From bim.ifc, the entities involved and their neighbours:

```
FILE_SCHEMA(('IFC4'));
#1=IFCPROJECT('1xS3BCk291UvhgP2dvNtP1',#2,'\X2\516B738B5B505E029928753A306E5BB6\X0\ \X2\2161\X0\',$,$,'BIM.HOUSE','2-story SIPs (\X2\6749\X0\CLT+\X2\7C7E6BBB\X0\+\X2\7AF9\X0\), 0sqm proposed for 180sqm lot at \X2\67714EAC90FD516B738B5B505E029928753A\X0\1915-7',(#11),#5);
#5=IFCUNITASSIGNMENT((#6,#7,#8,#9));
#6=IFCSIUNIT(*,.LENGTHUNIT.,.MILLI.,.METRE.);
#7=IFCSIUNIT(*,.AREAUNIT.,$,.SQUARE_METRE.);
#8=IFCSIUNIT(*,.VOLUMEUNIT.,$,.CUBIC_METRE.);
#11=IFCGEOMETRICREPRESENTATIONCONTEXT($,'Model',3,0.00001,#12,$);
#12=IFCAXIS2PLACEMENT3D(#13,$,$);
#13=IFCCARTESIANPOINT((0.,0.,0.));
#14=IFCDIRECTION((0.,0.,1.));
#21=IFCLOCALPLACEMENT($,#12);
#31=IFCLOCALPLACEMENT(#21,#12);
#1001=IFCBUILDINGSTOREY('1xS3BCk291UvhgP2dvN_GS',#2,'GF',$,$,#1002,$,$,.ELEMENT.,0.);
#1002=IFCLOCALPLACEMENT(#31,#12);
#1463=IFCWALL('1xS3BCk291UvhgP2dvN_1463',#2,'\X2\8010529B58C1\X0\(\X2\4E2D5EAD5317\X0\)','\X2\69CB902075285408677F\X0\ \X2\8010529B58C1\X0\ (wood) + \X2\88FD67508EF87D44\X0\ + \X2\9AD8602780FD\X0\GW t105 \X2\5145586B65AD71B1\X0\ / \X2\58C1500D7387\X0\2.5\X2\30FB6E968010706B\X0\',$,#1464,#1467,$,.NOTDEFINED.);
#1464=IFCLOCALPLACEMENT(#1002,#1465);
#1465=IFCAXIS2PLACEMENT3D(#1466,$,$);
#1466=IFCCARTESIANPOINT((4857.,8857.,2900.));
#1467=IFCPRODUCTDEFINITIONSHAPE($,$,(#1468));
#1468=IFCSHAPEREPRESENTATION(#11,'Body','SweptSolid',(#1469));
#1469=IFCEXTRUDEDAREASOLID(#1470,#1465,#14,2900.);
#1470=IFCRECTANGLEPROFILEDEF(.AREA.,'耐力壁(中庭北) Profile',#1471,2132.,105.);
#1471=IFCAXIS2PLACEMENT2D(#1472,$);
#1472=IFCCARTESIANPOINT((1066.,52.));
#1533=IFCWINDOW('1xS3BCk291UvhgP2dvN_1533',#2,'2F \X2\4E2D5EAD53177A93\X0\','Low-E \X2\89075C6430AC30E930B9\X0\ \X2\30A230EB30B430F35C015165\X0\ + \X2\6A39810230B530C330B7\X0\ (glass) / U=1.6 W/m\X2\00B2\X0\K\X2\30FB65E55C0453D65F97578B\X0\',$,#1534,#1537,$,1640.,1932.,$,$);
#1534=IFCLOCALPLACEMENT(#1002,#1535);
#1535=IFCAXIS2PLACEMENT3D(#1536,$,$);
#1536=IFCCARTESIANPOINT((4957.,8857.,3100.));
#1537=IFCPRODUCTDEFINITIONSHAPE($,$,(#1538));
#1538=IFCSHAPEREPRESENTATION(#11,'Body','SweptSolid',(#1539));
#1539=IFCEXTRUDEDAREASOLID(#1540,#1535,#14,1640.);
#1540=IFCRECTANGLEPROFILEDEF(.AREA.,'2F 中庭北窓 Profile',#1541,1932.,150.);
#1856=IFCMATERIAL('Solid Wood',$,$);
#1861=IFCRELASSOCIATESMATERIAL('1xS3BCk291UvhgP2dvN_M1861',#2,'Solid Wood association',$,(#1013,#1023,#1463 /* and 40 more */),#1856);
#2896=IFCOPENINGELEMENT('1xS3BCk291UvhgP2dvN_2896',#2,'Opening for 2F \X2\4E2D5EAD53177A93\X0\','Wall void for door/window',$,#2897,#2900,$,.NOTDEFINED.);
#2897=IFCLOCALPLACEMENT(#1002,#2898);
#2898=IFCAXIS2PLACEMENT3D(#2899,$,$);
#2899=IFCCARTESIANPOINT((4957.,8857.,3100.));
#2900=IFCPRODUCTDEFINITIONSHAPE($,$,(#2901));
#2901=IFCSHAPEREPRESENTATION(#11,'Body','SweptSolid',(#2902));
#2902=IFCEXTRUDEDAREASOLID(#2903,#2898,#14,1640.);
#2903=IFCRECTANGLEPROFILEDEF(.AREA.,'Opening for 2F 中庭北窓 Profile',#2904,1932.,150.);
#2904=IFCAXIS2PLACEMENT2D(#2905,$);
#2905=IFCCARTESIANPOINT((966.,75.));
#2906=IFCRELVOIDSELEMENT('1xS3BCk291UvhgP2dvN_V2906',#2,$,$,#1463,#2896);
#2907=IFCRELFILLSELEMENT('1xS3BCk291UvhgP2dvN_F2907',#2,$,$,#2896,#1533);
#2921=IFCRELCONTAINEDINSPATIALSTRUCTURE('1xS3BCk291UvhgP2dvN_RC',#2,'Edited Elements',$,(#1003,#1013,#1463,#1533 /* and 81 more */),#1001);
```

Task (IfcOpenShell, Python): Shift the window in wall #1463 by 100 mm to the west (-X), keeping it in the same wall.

```python
import ifcopenshell
import ifcopenshell.api.geometry
import ifcopenshell.util.placement

model = ifcopenshell.open("bim.ifc")

window = model.by_guid("1xS3BCk291UvhgP2dvN_1533")
opening = window.FillsVoids[0].RelatingOpeningElement
wall = opening.VoidsElements[0].RelatingBuildingElement

wall_matrix = ifcopenshell.util.placement.get_local_placement(wall.ObjectPlacement)
shift = wall_matrix[:3, 0] * -100.0
before = ifcopenshell.util.placement.get_local_placement(window.ObjectPlacement)[:3, 3].copy()

# The window is not placed relative to its opening, so move both.
for product in (opening, window):
    matrix = ifcopenshell.util.placement.get_local_placement(product.ObjectPlacement)
    matrix[:3, 3] += shift
    ifcopenshell.api.geometry.edit_object_placement(model, product=product, matrix=matrix, is_si=False)

after = ifcopenshell.util.placement.get_local_placement(window.ObjectPlacement)[:3, 3]
print("window moved by", (after - before).round(3) + 0.0)

model.write("bim_v2.ifc")
```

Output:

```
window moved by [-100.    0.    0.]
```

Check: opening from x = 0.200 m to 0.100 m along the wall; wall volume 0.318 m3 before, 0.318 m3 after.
